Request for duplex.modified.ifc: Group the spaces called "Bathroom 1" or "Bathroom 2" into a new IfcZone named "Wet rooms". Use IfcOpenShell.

First a look at what the model holds.

```python
import ifcopenshell

model = ifcopenshell.open("duplex.modified.ifc")
print(model.schema)
seen = {}
for space in model.by_type("IfcSpace"):
    seen[space.LongName] = seen.get(space.LongName, 0) + 1
for name, count in sorted(seen.items(), key=str):
    print(count, "x", name)
print("zones:", [z.Name for z in model.by_type("IfcZone")][:20])
```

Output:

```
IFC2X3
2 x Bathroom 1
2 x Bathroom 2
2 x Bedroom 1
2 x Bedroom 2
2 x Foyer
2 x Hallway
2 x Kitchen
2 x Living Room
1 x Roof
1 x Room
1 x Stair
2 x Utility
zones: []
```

```python
import ifcopenshell
import ifcopenshell.api.group
import ifcopenshell.api.root

model = ifcopenshell.open("duplex.modified.ifc")

names = {"Bathroom 1", "Bathroom 2"}
spaces = [s for s in model.by_type("IfcSpace") if s.LongName in names]

zone = ifcopenshell.api.root.create_entity(model, ifc_class="IfcZone", name="Wet rooms")
ifcopenshell.api.group.assign_group(model, products=spaces, group=zone)
print(len(spaces), "spaces in", zone.Name)

model.write("duplex.modified_updated.ifc")
```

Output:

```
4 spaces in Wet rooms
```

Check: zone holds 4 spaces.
